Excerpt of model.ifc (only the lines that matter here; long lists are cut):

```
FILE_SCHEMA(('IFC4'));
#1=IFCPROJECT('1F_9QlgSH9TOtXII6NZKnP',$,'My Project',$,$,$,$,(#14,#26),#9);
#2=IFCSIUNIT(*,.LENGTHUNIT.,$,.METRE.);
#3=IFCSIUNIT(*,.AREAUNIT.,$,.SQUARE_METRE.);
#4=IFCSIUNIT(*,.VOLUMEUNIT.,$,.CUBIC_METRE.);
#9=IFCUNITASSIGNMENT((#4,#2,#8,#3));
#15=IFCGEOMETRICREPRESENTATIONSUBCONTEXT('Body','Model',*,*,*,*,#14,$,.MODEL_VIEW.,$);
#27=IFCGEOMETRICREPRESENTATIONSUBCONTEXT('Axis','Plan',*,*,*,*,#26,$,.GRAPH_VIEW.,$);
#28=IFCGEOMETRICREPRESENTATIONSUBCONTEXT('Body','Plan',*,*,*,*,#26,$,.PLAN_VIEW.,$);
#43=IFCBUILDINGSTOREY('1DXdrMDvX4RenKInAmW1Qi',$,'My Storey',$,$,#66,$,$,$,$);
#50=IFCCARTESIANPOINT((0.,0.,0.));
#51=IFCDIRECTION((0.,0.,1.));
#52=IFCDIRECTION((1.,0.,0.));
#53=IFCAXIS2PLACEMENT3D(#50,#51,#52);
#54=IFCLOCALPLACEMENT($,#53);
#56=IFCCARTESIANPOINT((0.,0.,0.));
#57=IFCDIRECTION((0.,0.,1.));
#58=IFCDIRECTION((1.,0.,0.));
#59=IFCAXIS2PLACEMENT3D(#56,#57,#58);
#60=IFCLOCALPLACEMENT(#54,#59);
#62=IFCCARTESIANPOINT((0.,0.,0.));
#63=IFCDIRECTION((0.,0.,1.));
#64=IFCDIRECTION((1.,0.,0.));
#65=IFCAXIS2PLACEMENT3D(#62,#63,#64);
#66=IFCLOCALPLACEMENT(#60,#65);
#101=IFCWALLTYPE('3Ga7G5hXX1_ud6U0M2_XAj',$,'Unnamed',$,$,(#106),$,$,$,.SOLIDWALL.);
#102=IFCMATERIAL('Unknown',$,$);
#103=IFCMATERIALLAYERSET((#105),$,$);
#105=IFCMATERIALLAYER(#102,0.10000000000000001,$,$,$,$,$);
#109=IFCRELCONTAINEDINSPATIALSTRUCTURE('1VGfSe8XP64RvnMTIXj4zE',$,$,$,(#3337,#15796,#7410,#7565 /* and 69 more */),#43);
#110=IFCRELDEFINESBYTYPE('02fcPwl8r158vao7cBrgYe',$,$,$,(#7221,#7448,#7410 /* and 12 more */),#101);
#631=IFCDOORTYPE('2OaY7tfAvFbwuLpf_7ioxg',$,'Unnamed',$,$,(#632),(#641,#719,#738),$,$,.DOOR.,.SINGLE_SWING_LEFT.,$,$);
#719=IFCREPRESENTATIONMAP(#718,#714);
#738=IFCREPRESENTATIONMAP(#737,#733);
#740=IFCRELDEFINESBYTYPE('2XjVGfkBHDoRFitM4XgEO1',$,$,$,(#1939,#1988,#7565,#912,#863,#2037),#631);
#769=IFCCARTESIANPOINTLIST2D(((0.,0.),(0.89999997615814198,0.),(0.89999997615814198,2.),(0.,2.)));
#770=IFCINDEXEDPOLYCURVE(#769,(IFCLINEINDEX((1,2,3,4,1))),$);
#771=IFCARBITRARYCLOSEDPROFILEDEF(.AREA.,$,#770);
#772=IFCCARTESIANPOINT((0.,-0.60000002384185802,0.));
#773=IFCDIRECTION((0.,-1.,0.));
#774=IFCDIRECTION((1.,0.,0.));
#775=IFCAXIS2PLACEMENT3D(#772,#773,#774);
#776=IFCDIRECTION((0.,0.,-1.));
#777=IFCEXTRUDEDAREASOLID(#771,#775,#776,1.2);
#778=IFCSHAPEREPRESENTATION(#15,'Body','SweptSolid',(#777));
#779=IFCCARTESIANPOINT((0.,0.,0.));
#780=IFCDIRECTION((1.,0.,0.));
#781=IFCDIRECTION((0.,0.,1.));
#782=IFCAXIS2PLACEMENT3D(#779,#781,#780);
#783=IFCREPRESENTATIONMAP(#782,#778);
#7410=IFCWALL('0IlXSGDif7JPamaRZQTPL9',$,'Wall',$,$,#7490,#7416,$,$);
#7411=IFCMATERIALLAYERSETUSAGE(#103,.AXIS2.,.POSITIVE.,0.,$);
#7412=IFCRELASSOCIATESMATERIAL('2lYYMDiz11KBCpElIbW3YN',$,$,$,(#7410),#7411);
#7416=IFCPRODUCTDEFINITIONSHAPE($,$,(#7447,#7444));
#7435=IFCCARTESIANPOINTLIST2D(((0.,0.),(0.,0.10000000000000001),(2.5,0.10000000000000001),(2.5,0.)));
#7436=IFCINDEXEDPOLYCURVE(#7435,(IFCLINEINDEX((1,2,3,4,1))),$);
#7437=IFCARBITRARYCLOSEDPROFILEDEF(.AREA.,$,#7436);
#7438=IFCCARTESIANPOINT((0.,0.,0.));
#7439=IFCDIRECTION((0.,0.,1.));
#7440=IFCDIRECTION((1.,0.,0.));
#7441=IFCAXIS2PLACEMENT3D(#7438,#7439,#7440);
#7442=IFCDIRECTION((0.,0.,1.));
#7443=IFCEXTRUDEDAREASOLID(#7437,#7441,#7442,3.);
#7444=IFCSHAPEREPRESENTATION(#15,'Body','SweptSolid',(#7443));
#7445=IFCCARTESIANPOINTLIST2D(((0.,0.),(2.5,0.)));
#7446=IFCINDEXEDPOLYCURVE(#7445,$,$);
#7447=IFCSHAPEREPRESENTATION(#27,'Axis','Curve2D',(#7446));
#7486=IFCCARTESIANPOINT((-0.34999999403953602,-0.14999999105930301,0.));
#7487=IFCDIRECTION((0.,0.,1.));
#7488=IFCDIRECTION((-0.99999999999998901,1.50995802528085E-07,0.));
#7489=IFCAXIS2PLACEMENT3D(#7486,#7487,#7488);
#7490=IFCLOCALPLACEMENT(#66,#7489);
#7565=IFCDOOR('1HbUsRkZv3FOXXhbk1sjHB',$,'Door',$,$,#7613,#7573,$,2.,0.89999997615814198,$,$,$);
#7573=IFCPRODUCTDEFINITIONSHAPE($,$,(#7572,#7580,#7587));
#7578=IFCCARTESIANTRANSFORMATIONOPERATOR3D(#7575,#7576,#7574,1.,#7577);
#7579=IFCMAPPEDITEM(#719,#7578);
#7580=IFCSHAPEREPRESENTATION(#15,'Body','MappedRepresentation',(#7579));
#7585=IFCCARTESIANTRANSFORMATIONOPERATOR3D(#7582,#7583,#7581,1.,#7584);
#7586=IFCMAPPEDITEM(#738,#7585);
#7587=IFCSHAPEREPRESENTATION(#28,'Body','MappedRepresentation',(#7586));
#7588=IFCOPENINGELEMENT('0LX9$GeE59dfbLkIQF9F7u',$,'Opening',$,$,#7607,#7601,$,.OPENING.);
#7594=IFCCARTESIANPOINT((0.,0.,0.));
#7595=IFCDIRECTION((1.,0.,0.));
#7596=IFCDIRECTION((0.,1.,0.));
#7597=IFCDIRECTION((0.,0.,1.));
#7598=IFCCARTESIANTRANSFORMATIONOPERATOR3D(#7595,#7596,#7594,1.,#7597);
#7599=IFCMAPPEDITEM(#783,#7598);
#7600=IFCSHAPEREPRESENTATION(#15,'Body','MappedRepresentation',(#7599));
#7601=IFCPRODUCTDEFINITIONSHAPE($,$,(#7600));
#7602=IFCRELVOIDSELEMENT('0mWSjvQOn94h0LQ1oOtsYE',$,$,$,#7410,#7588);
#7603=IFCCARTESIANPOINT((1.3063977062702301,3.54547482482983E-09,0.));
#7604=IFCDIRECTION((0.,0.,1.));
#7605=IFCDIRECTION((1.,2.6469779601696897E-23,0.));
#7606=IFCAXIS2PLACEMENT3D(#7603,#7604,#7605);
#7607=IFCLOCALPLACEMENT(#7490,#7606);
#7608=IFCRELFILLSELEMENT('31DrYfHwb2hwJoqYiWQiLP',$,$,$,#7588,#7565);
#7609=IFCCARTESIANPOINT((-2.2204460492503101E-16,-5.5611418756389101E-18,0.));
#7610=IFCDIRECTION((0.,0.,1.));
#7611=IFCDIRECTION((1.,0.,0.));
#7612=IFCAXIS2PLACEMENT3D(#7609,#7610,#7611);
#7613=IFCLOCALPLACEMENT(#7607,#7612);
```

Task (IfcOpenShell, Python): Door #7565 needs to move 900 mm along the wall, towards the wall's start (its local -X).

```python
import ifcopenshell
import ifcopenshell.api.geometry
import ifcopenshell.util.placement
import ifcopenshell.util.unit

model = ifcopenshell.open("model.ifc")
unit_scale = ifcopenshell.util.unit.calculate_unit_scale(model)

door = model.by_guid("1HbUsRkZv3FOXXhbk1sjHB")
opening = door.FillsVoids[0].RelatingOpeningElement
wall = opening.VoidsElements[0].RelatingBuildingElement

wall_matrix = ifcopenshell.util.placement.get_local_placement(wall.ObjectPlacement)
shift = wall_matrix[:3, 0] * -0.9 / unit_scale
before = ifcopenshell.util.placement.get_local_placement(door.ObjectPlacement)[:3, 3].copy()

# The door is placed relative to its opening, so it follows when the opening moves.
matrix = ifcopenshell.util.placement.get_local_placement(opening.ObjectPlacement)
matrix[:3, 3] += shift
ifcopenshell.api.geometry.edit_object_placement(
    model, product=opening, matrix=matrix, is_si=False, should_transform_children=True
)

after = ifcopenshell.util.placement.get_local_placement(door.ObjectPlacement)[:3, 3]
print("door moved by", (after - before).round(3) + 0.0)

model.write("model_updated.ifc")
```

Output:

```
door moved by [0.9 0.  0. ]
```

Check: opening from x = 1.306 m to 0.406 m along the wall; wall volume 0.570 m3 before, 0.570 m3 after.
